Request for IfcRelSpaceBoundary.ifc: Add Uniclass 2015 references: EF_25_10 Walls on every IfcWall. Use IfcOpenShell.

First a look at what the model holds.

```python
import ifcopenshell

model = ifcopenshell.open("IfcRelSpaceBoundary.ifc")
print(model.schema)
print("classifications:", [c.Name for c in model.by_type("IfcClassification")])
for ifc_class in ("IfcDoor", "IfcRoof", "IfcStair", "IfcWall", "IfcWindow"):
    print(ifc_class, len(model.by_type(ifc_class)))
```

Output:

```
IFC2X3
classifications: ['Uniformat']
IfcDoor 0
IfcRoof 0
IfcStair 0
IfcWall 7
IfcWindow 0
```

```python
import ifcopenshell
import ifcopenshell.api.classification

model = ifcopenshell.open("IfcRelSpaceBoundary.ifc")

# IFC2X3 requires Source and Edition and has no link from the project to the system.
system = model.create_entity("IfcClassification", Source="NBS", Edition="2015", Name="Uniclass 2015")

codes = {
    "IfcWall": ("EF_25_10", "Walls"),
}
for ifc_class, (code, name) in codes.items():
    products = model.by_type(ifc_class)
    ifcopenshell.api.classification.add_reference(
        model, products=products, classification=system, identification=code, name=name
    )
    print(code, len(products))

model.write("IfcRelSpaceBoundary_updated.ifc")
```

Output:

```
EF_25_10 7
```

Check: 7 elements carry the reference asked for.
